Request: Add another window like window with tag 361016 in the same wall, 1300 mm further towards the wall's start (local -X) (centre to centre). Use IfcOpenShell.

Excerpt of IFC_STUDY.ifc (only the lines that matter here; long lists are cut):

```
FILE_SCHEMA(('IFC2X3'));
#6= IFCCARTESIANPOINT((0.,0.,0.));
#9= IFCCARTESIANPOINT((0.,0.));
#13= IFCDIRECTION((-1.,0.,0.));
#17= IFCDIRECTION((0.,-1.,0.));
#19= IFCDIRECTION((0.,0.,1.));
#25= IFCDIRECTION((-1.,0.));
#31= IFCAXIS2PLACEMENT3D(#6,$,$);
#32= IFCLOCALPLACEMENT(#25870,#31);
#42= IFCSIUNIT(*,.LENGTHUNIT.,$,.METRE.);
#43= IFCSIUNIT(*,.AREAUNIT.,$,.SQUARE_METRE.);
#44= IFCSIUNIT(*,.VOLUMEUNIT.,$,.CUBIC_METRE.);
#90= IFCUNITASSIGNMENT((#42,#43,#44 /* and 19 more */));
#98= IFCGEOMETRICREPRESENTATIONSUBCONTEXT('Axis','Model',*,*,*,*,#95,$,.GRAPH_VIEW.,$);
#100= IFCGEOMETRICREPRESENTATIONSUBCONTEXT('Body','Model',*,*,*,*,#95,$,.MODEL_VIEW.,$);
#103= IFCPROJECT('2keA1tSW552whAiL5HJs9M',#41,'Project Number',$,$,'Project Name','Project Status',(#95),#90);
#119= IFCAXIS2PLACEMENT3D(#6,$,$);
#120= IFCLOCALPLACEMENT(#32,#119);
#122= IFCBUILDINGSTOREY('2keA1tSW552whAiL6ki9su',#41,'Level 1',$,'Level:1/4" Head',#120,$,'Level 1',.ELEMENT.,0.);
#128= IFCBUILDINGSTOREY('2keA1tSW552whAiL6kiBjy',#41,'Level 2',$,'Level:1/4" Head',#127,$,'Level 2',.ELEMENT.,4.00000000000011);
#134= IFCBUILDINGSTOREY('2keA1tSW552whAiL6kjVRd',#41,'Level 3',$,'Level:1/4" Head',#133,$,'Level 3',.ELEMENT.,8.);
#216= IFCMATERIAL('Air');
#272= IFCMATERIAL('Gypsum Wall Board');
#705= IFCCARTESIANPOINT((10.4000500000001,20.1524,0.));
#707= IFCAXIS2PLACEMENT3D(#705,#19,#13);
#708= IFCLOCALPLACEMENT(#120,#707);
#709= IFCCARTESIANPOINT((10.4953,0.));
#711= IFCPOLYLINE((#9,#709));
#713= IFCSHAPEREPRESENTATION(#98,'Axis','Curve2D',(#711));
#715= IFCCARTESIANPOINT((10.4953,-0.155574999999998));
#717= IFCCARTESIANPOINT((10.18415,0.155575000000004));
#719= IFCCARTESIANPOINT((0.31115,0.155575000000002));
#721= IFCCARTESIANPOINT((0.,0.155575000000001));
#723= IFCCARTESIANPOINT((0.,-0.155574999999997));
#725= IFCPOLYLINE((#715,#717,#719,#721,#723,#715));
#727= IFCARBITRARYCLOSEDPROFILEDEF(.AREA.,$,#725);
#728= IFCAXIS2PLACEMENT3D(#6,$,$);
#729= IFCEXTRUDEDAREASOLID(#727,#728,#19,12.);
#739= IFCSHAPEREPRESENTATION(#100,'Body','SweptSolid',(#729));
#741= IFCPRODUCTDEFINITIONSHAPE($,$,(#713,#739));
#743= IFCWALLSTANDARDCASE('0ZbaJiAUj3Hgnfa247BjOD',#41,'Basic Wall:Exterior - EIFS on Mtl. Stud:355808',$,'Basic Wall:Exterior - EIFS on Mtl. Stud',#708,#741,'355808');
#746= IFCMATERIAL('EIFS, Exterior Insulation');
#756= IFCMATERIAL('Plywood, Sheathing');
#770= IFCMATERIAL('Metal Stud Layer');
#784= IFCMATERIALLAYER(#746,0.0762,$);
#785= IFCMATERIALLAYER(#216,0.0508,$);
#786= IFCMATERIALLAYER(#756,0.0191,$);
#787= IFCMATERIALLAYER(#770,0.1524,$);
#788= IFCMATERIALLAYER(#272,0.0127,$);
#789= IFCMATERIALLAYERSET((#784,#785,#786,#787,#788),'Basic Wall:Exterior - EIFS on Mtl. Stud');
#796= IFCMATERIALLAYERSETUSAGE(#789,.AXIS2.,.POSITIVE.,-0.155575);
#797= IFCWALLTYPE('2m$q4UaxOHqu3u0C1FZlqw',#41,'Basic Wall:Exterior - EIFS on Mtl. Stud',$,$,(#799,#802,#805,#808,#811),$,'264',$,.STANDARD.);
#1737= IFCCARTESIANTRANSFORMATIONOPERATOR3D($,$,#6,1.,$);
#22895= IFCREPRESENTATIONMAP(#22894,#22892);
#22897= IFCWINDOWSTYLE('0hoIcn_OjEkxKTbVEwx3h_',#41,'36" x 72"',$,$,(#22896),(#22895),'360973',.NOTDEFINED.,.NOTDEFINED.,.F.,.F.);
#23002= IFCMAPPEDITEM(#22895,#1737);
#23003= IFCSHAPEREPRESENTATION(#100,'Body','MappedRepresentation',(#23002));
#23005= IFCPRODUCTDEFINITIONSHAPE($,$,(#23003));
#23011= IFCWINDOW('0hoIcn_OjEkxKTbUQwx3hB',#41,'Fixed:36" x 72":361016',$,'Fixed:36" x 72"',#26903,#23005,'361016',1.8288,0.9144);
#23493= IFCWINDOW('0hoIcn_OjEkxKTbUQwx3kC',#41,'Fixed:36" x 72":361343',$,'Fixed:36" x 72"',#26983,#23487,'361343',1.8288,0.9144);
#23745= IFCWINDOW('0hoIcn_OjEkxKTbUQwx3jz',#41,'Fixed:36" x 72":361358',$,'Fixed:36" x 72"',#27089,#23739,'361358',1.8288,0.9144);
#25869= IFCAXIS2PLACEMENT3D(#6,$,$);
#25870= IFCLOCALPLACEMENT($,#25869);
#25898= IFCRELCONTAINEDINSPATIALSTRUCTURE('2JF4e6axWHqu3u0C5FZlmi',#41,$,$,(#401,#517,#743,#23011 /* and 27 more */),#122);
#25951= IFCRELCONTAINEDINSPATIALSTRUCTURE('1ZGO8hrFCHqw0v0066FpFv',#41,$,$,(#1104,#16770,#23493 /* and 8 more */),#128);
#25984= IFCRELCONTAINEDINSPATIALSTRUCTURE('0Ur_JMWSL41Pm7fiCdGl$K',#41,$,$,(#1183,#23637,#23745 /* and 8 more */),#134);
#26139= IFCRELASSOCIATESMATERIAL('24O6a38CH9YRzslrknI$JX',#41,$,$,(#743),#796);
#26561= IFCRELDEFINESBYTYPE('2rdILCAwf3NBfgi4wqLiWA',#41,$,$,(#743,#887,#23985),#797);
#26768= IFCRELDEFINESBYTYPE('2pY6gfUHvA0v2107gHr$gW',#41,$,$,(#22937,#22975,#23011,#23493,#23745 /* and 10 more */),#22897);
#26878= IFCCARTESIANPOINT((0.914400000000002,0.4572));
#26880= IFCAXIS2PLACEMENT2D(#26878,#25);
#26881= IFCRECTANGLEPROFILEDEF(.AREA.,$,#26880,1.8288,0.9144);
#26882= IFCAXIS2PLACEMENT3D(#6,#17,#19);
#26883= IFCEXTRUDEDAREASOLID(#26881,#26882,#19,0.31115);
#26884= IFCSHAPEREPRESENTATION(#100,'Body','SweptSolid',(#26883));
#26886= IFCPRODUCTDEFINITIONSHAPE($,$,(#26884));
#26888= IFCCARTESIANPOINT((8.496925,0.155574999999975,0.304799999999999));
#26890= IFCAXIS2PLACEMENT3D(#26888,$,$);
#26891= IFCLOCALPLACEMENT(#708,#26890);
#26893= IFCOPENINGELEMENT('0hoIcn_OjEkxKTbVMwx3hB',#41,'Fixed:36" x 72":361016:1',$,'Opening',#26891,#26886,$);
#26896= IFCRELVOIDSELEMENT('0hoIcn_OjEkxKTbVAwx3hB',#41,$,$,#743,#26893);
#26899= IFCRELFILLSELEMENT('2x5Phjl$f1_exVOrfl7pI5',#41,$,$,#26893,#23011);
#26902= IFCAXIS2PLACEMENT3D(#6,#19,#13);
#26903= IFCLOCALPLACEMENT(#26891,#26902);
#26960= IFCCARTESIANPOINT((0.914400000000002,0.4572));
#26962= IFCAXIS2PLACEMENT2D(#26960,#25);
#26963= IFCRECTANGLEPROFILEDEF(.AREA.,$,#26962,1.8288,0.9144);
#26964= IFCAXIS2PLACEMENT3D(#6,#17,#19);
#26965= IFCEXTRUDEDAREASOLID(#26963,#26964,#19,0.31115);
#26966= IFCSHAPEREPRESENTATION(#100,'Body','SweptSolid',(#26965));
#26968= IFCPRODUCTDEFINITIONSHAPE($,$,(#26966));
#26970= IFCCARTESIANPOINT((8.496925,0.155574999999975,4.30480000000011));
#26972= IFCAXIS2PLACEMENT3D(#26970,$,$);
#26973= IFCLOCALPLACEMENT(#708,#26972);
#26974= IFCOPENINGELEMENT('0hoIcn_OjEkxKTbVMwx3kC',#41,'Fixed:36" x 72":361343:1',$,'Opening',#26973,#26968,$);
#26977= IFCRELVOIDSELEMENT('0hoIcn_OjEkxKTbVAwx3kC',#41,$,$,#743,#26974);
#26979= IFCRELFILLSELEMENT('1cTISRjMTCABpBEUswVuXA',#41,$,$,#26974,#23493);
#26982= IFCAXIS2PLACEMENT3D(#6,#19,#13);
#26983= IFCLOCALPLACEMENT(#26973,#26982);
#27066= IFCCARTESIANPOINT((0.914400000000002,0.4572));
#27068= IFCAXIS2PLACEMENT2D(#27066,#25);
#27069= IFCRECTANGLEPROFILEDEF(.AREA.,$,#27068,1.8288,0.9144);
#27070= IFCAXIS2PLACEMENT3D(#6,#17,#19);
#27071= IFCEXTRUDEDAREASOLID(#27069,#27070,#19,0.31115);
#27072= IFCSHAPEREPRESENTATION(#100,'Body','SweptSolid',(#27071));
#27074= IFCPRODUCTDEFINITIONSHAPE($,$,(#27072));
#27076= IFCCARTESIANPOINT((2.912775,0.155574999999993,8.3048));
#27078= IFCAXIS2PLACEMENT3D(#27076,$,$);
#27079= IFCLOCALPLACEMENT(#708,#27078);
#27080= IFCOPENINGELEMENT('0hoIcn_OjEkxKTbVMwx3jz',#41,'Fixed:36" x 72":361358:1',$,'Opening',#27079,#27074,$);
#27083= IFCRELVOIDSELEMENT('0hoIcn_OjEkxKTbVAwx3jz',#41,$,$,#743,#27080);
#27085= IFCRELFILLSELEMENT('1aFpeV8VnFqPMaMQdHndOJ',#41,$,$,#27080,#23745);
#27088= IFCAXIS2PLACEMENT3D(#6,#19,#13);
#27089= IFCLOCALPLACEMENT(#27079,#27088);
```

```python
import ifcopenshell
import ifcopenshell.api.feature
import ifcopenshell.api.geometry
import ifcopenshell.api.root
import ifcopenshell.geom
import ifcopenshell.util.element
import ifcopenshell.util.placement
import ifcopenshell.util.shape
import ifcopenshell.util.unit

model = ifcopenshell.open("IFC_STUDY.ifc")
unit_scale = ifcopenshell.util.unit.calculate_unit_scale(model)
settings = ifcopenshell.geom.settings()


def volume(element):
    """Net volume in cubic metres, openings subtracted."""
    shape = ifcopenshell.geom.create_shape(settings, element)
    return ifcopenshell.util.shape.get_volume(shape.geometry)


def reuse_history(source, copy):
    """copy_class also copies each property set's owner history, people and application; keep the originals."""
    for rel in copy.IsDefinedBy:
        if rel.is_a("IfcRelDefinesByProperties") and (history := rel.RelatingPropertyDefinition.OwnerHistory):
            rel.RelatingPropertyDefinition.OwnerHistory = source.OwnerHistory
            ifcopenshell.util.element.remove_deep2(model, history)


window = model.by_guid("0hoIcn_OjEkxKTbUQwx3hB")
opening = window.FillsVoids[0].RelatingOpeningElement
wall = opening.VoidsElements[0].RelatingBuildingElement
before = volume(wall)
shift = ifcopenshell.util.placement.get_local_placement(wall.ObjectPlacement)[:3, 0] * -1.3 / unit_scale

# copy_class copies the void relationship, type, container and properties, but no geometry.
new_opening = ifcopenshell.api.root.copy_class(model, product=opening)
new_opening.Representation = ifcopenshell.util.element.copy_deep(
    model, opening.Representation, exclude=["IfcGeometricRepresentationContext", "IfcRepresentationMap"]
)
new_opening.Name = 'Fixed:36" x 72"'
new_window = ifcopenshell.api.root.copy_class(model, product=window)
new_window.Representation = ifcopenshell.util.element.copy_deep(
    model, window.Representation, exclude=["IfcGeometricRepresentationContext", "IfcRepresentationMap"]
)
new_window.Name = 'Fixed:36" x 72"'
new_window.Tag = None
reuse_history(window, new_window)
fills = ifcopenshell.api.feature.add_filling(model, opening=new_opening, element=new_window)
fills.OwnerHistory = new_window.OwnerHistory  # required in IFC2X3

for old, new in ((opening, new_opening), (window, new_window)):
    matrix = ifcopenshell.util.placement.get_local_placement(old.ObjectPlacement)
    matrix[:3, 3] += shift
    ifcopenshell.api.geometry.edit_object_placement(model, product=new, matrix=matrix, is_si=False)

after = volume(wall)

print(f"wall volume {before:.3f} -> {after:.3f} m3")

model.write("IFC_STUDY-out.ifc")
```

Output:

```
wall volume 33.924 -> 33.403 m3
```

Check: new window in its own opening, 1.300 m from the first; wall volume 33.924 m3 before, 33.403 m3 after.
